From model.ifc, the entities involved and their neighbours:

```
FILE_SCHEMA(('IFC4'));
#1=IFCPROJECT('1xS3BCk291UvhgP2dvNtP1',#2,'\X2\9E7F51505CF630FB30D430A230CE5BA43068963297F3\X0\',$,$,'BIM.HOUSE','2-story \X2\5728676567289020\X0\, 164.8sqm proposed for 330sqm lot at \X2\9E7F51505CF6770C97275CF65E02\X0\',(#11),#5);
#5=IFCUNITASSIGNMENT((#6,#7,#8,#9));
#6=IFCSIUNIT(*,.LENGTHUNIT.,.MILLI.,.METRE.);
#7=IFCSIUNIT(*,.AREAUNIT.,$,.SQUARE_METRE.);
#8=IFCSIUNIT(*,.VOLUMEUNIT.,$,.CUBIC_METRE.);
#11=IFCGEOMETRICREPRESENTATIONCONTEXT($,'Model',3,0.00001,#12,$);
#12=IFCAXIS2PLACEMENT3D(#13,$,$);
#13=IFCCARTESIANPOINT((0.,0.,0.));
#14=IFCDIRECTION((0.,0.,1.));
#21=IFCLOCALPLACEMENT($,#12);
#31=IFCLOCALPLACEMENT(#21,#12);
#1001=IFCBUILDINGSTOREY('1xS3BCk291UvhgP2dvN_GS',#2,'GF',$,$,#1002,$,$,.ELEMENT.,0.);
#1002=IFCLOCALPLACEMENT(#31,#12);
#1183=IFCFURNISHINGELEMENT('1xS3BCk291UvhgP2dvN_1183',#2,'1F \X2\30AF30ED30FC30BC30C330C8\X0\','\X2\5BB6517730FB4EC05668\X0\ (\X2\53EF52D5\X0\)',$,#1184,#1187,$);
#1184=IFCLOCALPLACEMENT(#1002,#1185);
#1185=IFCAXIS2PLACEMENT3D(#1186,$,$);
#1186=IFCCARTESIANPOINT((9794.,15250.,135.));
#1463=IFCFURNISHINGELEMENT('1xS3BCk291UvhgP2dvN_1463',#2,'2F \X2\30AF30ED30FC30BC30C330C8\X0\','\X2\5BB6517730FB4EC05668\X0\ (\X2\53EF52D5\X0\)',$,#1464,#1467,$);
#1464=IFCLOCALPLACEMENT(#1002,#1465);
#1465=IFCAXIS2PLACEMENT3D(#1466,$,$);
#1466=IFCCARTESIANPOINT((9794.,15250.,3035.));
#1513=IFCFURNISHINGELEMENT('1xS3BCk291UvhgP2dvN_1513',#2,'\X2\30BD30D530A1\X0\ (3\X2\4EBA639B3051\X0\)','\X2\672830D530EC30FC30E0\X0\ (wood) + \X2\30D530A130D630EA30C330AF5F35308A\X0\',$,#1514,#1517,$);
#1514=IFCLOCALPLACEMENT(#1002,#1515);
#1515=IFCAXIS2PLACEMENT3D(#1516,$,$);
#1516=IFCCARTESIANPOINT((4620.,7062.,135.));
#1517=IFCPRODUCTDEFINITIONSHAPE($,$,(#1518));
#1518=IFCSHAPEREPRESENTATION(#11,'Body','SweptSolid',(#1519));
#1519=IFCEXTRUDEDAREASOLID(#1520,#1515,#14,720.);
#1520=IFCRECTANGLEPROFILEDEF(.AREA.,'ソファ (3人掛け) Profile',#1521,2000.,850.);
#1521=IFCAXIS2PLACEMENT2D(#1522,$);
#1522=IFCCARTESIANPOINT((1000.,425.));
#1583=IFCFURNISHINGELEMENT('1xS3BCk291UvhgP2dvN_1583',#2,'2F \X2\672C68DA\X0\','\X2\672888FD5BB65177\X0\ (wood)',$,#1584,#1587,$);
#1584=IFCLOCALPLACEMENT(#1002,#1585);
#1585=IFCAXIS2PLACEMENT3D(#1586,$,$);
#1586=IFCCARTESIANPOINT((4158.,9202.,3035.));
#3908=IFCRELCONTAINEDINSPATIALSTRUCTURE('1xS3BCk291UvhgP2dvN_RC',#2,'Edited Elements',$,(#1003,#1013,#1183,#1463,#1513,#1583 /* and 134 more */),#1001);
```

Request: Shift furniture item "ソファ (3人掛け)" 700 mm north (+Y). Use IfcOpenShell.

```python
import ifcopenshell
import ifcopenshell.api.geometry
import ifcopenshell.util.placement
import ifcopenshell.util.unit

model = ifcopenshell.open("model.ifc")
unit_scale = ifcopenshell.util.unit.calculate_unit_scale(model)

item = model.by_guid("1xS3BCk291UvhgP2dvN_1513")
matrix = ifcopenshell.util.placement.get_local_placement(item.ObjectPlacement)
matrix[1, 3] += 0.7 / unit_scale
ifcopenshell.api.geometry.edit_object_placement(model, product=item, matrix=matrix, is_si=False)

print(ifcopenshell.util.placement.get_local_placement(item.ObjectPlacement).round(3) + 0.0)

model.write("model_rev.ifc")
```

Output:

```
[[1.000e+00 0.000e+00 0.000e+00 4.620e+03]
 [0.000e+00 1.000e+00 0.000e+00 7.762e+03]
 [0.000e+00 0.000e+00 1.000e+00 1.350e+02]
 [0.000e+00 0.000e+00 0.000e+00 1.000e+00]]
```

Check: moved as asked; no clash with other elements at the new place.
